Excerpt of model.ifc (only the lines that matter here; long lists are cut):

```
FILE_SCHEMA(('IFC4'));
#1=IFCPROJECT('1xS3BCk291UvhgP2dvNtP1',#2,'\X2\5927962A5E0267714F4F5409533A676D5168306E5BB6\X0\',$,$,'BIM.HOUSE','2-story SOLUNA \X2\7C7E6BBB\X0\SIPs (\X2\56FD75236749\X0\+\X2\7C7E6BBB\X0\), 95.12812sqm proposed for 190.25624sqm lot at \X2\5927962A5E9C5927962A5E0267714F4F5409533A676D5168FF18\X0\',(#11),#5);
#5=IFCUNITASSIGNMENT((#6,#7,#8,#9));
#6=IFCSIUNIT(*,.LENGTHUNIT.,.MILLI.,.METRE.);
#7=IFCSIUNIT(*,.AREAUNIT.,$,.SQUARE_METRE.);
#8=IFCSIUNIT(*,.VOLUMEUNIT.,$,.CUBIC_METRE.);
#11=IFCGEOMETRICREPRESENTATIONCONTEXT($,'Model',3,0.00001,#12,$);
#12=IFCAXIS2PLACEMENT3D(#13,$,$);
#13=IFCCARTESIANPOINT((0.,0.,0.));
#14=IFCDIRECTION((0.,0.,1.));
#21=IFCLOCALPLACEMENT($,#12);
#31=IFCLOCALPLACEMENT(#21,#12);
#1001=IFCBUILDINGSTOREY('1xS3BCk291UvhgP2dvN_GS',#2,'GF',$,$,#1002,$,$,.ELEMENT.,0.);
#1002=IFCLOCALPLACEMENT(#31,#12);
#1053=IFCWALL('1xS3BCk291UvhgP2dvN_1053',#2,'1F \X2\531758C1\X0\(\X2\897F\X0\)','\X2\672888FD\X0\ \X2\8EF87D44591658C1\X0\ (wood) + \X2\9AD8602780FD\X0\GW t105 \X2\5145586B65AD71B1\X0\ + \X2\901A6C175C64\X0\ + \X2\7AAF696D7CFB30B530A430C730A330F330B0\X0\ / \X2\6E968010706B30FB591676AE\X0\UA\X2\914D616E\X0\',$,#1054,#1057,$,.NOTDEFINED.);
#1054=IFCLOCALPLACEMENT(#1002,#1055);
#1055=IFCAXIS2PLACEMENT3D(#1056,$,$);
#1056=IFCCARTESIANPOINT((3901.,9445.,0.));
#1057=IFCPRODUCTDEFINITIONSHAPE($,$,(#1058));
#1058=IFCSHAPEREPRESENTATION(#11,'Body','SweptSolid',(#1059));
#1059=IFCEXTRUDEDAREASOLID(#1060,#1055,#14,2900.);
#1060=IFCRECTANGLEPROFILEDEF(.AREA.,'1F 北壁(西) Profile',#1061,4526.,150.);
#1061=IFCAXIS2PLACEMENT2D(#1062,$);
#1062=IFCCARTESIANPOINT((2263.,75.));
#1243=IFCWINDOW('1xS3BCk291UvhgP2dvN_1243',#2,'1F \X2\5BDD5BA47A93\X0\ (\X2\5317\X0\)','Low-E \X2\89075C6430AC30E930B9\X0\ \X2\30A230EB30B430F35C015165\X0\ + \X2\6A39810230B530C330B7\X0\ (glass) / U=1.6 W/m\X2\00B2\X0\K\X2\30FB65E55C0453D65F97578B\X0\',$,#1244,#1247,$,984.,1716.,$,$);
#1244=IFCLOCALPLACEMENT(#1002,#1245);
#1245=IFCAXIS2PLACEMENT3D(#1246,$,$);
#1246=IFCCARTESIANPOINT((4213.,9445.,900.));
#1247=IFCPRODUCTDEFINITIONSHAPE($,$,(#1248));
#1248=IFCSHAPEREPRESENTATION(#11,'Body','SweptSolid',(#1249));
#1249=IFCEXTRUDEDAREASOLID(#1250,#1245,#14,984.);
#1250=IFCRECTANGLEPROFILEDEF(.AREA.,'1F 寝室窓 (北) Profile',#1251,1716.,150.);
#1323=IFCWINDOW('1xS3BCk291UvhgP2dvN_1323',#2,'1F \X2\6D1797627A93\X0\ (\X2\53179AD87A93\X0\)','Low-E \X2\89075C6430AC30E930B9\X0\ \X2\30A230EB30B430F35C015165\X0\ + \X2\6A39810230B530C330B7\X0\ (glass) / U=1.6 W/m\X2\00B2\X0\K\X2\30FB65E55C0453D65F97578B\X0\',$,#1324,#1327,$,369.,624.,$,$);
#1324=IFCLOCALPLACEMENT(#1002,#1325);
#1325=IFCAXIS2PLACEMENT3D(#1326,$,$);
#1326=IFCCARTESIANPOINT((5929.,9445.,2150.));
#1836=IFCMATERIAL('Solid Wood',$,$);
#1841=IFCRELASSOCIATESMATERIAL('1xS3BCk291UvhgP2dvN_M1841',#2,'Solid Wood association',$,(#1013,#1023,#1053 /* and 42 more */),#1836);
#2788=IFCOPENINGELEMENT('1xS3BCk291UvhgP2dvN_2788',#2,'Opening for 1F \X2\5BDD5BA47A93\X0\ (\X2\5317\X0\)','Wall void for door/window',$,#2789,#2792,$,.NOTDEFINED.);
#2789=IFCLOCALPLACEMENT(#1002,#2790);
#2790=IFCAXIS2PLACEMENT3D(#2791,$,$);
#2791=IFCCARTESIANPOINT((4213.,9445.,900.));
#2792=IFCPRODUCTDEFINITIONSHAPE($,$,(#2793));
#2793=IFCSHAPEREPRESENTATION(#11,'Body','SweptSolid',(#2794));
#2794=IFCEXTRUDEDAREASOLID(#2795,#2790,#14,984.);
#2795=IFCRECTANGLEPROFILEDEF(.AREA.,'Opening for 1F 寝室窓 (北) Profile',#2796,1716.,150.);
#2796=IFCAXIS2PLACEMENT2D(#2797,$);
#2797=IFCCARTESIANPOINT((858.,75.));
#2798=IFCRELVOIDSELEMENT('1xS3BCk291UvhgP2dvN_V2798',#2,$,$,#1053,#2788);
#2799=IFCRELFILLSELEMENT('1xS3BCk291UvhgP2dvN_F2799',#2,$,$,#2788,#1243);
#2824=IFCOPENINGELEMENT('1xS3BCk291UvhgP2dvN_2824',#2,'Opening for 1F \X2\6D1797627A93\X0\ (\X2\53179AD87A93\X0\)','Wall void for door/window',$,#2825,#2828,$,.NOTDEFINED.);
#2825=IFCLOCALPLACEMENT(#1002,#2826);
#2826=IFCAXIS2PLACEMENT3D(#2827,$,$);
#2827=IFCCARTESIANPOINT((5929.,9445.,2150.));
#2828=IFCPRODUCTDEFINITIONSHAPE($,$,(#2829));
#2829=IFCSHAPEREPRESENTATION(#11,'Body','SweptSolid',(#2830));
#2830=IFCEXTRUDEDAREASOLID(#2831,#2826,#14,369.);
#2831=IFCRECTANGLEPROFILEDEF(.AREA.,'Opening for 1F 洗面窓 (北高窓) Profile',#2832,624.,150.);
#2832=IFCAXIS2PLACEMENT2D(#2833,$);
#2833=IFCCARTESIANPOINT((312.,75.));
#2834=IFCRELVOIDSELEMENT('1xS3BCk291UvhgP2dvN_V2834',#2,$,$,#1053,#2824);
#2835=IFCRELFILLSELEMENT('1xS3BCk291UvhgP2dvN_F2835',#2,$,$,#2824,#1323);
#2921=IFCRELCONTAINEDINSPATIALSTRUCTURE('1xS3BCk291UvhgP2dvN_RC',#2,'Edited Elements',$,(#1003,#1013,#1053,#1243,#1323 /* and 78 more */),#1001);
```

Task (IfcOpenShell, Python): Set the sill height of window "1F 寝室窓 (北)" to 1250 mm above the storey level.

```python
import numpy as np
import ifcopenshell
import ifcopenshell.api.geometry
import ifcopenshell.geom
import ifcopenshell.util.element
import ifcopenshell.util.placement
import ifcopenshell.util.shape
import ifcopenshell.util.unit

model = ifcopenshell.open("model.ifc")
unit_scale = ifcopenshell.util.unit.calculate_unit_scale(model)

window = model.by_guid("1xS3BCk291UvhgP2dvN_1243")
opening = window.FillsVoids[0].RelatingOpeningElement
storey = ifcopenshell.util.element.get_container(window, ifc_class="IfcBuildingStorey")
level = ifcopenshell.util.placement.get_local_placement(storey.ObjectPlacement)[2, 3]

# The opening's origin need not be at the sill, so measure its lowest point.
shape = ifcopenshell.geom.create_shape(ifcopenshell.geom.settings(), opening)
bottom = ifcopenshell.util.shape.get_shape_bottom_elevation(shape, shape.geometry) / unit_scale
dz = level + 1.25 / unit_scale - bottom

shift = np.array([0.0, 0.0, dz])
# The window is not placed relative to its opening, so move both.
for product in (opening, window):
    matrix = ifcopenshell.util.placement.get_local_placement(product.ObjectPlacement)
    matrix[:3, 3] += shift
    ifcopenshell.api.geometry.edit_object_placement(model, product=product, matrix=matrix, is_si=False)

print(f"moved by {dz * unit_scale:+.3f} m")

model.write("model_v2.ifc")
```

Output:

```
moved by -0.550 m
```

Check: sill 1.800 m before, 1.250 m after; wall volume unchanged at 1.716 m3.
